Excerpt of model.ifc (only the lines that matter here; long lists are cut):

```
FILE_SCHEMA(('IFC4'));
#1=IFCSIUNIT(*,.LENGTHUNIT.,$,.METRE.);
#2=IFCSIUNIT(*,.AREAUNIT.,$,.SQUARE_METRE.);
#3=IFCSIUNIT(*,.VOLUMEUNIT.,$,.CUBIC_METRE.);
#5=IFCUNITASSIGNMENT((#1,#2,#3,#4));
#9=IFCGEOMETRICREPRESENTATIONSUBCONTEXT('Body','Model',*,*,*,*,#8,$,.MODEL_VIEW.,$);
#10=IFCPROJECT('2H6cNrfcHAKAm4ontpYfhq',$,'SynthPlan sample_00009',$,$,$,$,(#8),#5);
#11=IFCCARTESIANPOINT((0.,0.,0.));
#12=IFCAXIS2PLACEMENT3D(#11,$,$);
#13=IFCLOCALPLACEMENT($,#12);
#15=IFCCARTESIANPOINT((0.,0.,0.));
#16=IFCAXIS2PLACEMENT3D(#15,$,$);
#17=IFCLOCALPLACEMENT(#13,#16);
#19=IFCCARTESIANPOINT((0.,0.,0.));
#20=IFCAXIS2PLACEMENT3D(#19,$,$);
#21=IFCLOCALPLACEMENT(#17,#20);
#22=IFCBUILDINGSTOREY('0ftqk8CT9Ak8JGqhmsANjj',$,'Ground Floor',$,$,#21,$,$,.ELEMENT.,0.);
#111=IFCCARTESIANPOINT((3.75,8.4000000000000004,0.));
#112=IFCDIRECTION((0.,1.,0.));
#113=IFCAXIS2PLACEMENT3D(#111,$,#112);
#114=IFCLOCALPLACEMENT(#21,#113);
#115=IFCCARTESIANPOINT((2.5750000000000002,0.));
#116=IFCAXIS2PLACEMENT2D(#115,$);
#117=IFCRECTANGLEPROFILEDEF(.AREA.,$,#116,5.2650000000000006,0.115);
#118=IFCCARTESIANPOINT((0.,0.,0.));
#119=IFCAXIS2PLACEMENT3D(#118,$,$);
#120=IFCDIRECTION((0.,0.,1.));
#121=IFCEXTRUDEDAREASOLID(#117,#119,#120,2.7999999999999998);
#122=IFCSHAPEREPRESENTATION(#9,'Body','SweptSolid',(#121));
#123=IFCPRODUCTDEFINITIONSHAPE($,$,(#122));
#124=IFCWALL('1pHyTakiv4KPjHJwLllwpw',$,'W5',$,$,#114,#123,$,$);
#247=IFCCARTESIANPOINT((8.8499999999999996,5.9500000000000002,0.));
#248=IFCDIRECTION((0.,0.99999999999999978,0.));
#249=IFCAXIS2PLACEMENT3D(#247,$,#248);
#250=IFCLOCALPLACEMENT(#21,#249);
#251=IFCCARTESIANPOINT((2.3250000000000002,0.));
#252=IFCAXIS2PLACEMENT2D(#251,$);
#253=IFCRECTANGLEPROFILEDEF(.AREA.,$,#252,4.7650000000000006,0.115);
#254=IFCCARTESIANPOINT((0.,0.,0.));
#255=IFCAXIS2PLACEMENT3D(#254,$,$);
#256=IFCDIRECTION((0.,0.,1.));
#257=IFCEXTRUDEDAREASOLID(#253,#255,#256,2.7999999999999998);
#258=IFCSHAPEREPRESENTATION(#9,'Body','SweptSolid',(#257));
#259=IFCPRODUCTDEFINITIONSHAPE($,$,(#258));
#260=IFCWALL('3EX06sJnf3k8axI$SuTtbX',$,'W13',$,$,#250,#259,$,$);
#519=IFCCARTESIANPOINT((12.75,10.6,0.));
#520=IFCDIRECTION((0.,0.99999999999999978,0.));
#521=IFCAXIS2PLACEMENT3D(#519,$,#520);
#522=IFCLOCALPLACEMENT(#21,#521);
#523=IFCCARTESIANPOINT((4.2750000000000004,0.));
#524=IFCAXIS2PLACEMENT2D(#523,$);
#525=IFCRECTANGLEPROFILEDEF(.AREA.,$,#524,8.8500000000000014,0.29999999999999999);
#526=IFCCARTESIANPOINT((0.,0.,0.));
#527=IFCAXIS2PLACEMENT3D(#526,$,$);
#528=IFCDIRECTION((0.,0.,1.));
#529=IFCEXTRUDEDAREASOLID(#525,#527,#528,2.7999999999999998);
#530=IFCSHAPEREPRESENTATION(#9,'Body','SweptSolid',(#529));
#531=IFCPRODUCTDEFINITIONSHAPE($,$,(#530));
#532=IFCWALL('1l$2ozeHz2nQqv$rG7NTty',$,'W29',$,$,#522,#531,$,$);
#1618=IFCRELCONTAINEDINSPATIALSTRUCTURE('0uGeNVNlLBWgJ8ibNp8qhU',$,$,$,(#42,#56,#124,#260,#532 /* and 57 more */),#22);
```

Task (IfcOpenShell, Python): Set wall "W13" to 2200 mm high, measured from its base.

```python
import ifcopenshell
import ifcopenshell.geom
import ifcopenshell.util.representation
import ifcopenshell.util.shape
import ifcopenshell.util.unit

model = ifcopenshell.open("model.ifc")
unit_scale = ifcopenshell.util.unit.calculate_unit_scale(model)
settings = ifcopenshell.geom.settings()


def volume(element):
    """Net volume in cubic metres, openings subtracted."""
    shape = ifcopenshell.geom.create_shape(settings, element)
    return ifcopenshell.util.shape.get_volume(shape.geometry)


wall = model.by_id(260)
before = volume(wall)

body = ifcopenshell.util.representation.get_representation(wall, "Model", "Body")
solid = body.Items[0]
old_height = solid.Depth
solid.Depth = 2.2 / unit_scale
after = volume(wall)

print(f"height {old_height:g} -> {solid.Depth:g}, volume {before:.3f} -> {after:.3f} m3")

model.write("model_rev.ifc")
```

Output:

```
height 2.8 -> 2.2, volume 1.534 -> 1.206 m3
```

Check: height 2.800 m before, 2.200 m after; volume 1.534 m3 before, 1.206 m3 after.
